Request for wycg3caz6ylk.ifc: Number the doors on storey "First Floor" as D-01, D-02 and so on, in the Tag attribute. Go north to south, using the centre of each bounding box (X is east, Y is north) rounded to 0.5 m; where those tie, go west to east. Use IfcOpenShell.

First a look at what the model holds.

```python
import ifcopenshell
import ifcopenshell.util.element
import ifcopenshell.util.placement

model = ifcopenshell.open("wycg3caz6ylk.ifc")
print(model.schema)
storey = next(s for s in model.by_type("IfcBuildingStorey") if s.Name == "First Floor")
doors = [e for e in ifcopenshell.util.element.get_decomposition(storey) if e.is_a("IfcDoor")]
for e in sorted(doors, key=lambda e: e.id()):
    origin = ifcopenshell.util.placement.get_local_placement(e.ObjectPlacement)[:3, 3]
    print(e.id(), e.Tag, e.Name, origin.round(2) + 0.0, sep=" | ")
```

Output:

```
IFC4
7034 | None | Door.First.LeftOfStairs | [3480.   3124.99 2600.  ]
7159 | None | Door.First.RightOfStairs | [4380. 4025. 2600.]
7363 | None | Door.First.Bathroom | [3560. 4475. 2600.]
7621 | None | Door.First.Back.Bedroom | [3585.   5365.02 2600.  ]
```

```python
import ifcopenshell
import ifcopenshell.geom
import ifcopenshell.util.element
import ifcopenshell.util.shape

model = ifcopenshell.open("wycg3caz6ylk.ifc")
settings = ifcopenshell.geom.settings()
settings.set("use-world-coords", True)


def centre(element):
    shape = ifcopenshell.geom.create_shape(settings, element)
    return ifcopenshell.util.shape.get_bbox_centroid(shape.geometry)


storey = next(s for s in model.by_type("IfcBuildingStorey") if s.Name == "First Floor")
doors = [e for e in ifcopenshell.util.element.get_decomposition(storey) if e.is_a("IfcDoor")]

# Insertion points can sit at a corner or the storey origin, so sort by the geometry (in metres).
centres = {e: centre(e) for e in doors}
doors.sort(key=lambda e: (-round(centres[e][1] / 0.5), centres[e][0]))

for i, e in enumerate(doors, start=1):
    number = f"D-{i:02d}"
    e.Tag = number
    print(e.id(), number)

model.write("wycg3caz6ylk_edited.ifc")
```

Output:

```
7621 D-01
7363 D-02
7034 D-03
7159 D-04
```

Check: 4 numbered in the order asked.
